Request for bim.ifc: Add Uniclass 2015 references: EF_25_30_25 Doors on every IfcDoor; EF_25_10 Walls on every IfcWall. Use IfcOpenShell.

First a look at what the model holds.

```python
import ifcopenshell

model = ifcopenshell.open("bim.ifc")
print(model.schema)
print("classifications:", [c.Name for c in model.by_type("IfcClassification")])
for ifc_class in ("IfcDoor", "IfcRoof", "IfcStair", "IfcWall", "IfcWindow"):
    print(ifc_class, len(model.by_type(ifc_class)))
```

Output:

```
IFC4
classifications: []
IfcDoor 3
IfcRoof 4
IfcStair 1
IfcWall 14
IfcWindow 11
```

```python
import ifcopenshell
import ifcopenshell.api.classification

model = ifcopenshell.open("bim.ifc")

system = ifcopenshell.api.classification.add_classification(model, classification="Uniclass 2015")

codes = {
    "IfcDoor": ("EF_25_30_25", "Doors"),
    "IfcWall": ("EF_25_10", "Walls"),
}
for ifc_class, (code, name) in codes.items():
    products = model.by_type(ifc_class)
    ifcopenshell.api.classification.add_reference(
        model, products=products, classification=system, identification=code, name=name
    )
    print(code, len(products))

model.write("bim_edited.ifc")
```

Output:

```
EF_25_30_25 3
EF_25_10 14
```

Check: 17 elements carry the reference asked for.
